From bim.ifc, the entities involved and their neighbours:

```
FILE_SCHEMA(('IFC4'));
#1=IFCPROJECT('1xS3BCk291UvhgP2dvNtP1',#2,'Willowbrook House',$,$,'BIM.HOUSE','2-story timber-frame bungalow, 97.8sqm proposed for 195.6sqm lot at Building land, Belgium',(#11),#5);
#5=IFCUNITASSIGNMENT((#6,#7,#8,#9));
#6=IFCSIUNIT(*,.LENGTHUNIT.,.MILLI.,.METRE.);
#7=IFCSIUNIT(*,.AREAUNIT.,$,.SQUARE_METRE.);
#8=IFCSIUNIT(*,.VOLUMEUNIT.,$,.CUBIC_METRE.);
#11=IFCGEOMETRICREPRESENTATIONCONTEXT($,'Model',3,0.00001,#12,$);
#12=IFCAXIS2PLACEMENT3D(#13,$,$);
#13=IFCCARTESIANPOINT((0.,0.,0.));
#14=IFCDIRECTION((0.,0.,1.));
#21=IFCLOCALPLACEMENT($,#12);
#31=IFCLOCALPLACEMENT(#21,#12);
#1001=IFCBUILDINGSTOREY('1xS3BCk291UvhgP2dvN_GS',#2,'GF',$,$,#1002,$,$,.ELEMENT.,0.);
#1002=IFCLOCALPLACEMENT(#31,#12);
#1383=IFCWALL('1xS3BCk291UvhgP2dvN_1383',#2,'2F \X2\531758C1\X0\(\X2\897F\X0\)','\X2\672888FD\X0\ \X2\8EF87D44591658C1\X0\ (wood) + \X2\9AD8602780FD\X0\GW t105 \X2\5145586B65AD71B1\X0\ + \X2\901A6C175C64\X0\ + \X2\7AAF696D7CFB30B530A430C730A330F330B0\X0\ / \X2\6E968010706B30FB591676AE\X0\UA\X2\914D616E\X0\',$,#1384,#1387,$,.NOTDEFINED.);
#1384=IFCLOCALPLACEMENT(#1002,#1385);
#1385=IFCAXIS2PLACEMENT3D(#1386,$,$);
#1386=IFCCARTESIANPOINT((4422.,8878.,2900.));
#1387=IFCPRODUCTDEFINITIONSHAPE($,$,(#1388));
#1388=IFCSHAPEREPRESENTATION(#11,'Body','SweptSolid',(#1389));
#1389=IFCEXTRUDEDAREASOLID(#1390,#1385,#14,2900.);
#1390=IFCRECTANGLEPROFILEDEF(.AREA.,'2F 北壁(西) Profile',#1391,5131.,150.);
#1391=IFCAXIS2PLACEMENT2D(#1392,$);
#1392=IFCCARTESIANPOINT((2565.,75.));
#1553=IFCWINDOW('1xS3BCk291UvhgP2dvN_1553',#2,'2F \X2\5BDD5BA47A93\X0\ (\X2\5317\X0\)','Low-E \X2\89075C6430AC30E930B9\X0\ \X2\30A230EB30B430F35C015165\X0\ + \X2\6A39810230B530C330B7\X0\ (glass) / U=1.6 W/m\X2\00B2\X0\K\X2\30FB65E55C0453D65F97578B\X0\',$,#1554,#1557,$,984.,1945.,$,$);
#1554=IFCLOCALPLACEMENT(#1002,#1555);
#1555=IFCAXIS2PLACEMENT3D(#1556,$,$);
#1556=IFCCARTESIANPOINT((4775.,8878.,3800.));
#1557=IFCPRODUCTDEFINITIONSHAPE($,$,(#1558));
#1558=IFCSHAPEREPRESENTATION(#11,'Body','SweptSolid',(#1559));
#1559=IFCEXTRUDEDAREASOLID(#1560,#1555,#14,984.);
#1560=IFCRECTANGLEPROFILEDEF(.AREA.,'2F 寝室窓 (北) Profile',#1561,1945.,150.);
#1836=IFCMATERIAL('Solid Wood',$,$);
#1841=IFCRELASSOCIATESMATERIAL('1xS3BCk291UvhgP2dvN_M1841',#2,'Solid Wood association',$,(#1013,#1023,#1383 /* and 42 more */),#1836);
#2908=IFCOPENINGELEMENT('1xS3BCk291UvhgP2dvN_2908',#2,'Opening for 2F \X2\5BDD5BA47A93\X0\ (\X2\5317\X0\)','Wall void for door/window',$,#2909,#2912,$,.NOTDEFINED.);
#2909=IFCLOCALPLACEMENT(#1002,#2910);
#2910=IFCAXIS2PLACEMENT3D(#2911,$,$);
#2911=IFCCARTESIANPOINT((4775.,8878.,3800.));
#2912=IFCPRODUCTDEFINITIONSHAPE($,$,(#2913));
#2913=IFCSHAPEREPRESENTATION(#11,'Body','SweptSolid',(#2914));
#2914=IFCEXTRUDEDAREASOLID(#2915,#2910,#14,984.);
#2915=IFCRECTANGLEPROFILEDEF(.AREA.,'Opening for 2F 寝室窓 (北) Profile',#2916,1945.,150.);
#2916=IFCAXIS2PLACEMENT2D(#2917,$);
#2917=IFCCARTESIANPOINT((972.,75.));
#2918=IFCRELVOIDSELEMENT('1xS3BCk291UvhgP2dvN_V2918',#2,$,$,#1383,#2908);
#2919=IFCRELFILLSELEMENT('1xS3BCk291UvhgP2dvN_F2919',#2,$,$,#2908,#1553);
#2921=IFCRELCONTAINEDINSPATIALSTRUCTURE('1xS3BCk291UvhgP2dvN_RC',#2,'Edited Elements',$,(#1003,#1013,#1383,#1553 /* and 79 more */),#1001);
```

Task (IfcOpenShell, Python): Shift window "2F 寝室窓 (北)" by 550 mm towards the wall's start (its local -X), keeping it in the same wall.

```python
import ifcopenshell
import ifcopenshell.api.geometry
import ifcopenshell.util.placement

model = ifcopenshell.open("bim.ifc")

window = model.by_id(1553)
opening = window.FillsVoids[0].RelatingOpeningElement
wall = opening.VoidsElements[0].RelatingBuildingElement

wall_matrix = ifcopenshell.util.placement.get_local_placement(wall.ObjectPlacement)
shift = wall_matrix[:3, 0] * -550.0
before = ifcopenshell.util.placement.get_local_placement(window.ObjectPlacement)[:3, 3].copy()

# The window is not placed relative to its opening, so move both.
for product in (opening, window):
    matrix = ifcopenshell.util.placement.get_local_placement(product.ObjectPlacement)
    matrix[:3, 3] += shift
    ifcopenshell.api.geometry.edit_object_placement(model, product=product, matrix=matrix, is_si=False)

after = ifcopenshell.util.placement.get_local_placement(window.ObjectPlacement)[:3, 3]
print("window moved by", (after - before).round(3) + 0.0)

model.write("bim_updated.ifc")
```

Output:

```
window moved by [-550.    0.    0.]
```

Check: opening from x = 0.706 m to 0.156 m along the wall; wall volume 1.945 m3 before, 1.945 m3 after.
